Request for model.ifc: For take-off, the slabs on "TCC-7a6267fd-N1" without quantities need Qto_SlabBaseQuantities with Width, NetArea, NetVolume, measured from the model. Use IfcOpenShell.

First a look at what the model holds.

```python
import ifcopenshell
import ifcopenshell.util.element
import ifcopenshell.util.unit

model = ifcopenshell.open("model.ifc")
print(model.schema)
for unit_type in ("LENGTHUNIT", "AREAUNIT", "VOLUMEUNIT"):
    print(unit_type, ifcopenshell.util.unit.calculate_unit_scale(model, unit_type))
storey = next(s for s in model.by_type("IfcBuildingStorey") if s.Name == "TCC-7a6267fd-N1")
slabs = [e for e in ifcopenshell.util.element.get_decomposition(storey) if e.is_a("IfcSlab")]
for e in sorted(slabs, key=lambda e: e.id()):
    print(e.id(), e.is_a(), e.Name, list(ifcopenshell.util.element.get_psets(e, qtos_only=True)), sep=" | ")
```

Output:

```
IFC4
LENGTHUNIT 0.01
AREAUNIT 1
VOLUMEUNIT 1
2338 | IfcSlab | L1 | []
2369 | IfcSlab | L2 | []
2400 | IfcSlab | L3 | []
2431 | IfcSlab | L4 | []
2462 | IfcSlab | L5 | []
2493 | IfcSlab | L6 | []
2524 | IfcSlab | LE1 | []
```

```python
import ifcopenshell
import ifcopenshell.api.pset
import ifcopenshell.geom
import ifcopenshell.util.element
import ifcopenshell.util.shape
import ifcopenshell.util.unit

model = ifcopenshell.open("model.ifc")
unit_scale = ifcopenshell.util.unit.calculate_unit_scale(model)
area_scale = ifcopenshell.util.unit.calculate_unit_scale(model, "AREAUNIT")
volume_scale = ifcopenshell.util.unit.calculate_unit_scale(model, "VOLUMEUNIT")
settings = ifcopenshell.geom.settings()

storey = next(s for s in model.by_type("IfcBuildingStorey") if s.Name == "TCC-7a6267fd-N1")
slabs = [e for e in ifcopenshell.util.element.get_decomposition(storey) if e.is_a("IfcSlab")]

for e in sorted(slabs, key=lambda e: e.id()):
    if ifcopenshell.util.element.get_psets(e, qtos_only=True, should_inherit=False):
        continue
    # Geometry comes back in metres, in the element's own axes.
    shape = ifcopenshell.geom.create_shape(settings, e)
    values = {
        "Width": ifcopenshell.util.shape.get_z(shape.geometry) / unit_scale,
        "NetArea": ifcopenshell.util.shape.get_footprint_area(shape.geometry) / area_scale,
        "NetVolume": ifcopenshell.util.shape.get_volume(shape.geometry) / volume_scale,
    }
    qto = ifcopenshell.api.pset.add_qto(model, product=e, name="Qto_SlabBaseQuantities")
    ifcopenshell.api.pset.edit_qto(model, qto=qto, properties=values)
    print(e.id(), {k: round(v, 3) for k, v in values.items()})

model.write("model_rev.ifc")
```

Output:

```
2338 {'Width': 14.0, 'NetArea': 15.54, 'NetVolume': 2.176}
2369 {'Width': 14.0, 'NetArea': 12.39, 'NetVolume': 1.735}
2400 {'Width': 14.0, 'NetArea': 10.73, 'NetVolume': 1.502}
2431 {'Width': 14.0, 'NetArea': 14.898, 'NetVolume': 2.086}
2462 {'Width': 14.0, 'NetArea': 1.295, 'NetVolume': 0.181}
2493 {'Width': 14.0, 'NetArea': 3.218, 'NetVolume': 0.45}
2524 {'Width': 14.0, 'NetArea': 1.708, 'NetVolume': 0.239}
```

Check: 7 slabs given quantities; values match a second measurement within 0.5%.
